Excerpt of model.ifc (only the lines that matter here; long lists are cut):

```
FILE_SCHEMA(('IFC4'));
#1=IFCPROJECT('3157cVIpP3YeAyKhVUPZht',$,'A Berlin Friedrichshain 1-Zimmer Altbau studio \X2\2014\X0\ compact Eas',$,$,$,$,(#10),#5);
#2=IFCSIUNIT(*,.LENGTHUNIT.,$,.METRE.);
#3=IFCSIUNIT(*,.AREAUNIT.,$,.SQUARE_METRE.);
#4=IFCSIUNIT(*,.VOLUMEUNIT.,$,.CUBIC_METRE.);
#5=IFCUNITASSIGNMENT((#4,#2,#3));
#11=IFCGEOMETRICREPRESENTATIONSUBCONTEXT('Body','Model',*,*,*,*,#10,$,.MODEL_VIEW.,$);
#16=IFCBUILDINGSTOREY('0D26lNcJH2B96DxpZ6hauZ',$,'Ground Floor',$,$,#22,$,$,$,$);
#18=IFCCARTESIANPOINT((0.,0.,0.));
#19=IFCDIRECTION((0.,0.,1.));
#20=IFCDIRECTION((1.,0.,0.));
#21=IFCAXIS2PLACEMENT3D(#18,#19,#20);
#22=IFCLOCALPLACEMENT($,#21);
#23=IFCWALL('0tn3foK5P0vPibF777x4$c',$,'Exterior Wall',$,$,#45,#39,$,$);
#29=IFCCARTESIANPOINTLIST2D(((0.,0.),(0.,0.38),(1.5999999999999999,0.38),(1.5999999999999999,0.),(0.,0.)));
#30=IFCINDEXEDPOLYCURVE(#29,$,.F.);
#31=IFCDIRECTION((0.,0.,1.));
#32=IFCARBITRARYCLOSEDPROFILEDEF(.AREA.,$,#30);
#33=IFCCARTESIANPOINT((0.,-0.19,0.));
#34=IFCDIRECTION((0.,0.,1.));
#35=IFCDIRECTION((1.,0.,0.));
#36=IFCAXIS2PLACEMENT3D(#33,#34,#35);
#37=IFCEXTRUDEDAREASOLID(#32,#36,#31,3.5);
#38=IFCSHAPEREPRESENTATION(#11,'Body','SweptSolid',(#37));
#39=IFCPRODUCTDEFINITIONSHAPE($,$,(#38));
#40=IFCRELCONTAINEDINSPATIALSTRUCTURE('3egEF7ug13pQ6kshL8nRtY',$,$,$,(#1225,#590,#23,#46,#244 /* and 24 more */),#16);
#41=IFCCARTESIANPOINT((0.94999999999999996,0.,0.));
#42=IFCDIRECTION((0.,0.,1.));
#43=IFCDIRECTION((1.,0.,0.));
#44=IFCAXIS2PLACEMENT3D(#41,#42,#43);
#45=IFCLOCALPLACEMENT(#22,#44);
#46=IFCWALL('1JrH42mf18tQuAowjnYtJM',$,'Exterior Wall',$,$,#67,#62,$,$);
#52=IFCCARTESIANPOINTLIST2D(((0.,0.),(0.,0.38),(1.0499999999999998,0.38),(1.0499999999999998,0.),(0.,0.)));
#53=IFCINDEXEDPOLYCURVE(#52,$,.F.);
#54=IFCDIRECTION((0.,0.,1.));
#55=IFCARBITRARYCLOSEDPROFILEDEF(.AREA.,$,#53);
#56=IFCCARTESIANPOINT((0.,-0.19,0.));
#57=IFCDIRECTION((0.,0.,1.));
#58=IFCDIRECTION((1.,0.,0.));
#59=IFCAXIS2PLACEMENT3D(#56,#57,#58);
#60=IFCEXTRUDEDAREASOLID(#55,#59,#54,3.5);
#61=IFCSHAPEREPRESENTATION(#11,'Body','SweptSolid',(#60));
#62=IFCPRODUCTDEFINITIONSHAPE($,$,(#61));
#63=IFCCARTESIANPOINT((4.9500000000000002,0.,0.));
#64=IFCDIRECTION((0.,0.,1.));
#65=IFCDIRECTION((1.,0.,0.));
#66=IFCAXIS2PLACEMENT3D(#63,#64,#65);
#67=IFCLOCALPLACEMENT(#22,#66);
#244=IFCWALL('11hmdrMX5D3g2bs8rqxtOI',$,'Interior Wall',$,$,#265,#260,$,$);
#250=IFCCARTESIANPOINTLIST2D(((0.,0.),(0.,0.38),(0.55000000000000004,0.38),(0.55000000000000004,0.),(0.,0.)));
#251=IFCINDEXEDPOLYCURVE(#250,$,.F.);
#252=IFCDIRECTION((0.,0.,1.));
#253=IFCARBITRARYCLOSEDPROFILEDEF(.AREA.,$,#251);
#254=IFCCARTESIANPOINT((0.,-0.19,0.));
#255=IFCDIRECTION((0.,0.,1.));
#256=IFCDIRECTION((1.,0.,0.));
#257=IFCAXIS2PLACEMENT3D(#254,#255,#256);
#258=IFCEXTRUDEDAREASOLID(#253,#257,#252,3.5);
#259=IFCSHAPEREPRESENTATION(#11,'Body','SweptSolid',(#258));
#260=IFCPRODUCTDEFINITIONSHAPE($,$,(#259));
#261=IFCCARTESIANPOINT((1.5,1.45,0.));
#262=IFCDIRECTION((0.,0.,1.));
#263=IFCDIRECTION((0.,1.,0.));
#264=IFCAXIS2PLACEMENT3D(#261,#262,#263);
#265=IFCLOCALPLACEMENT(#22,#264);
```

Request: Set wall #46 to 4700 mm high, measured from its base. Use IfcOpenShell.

```python
import ifcopenshell
import ifcopenshell.geom
import ifcopenshell.util.representation
import ifcopenshell.util.shape
import ifcopenshell.util.unit

model = ifcopenshell.open("model.ifc")
unit_scale = ifcopenshell.util.unit.calculate_unit_scale(model)
settings = ifcopenshell.geom.settings()


def volume(element):
    """Net volume in cubic metres, openings subtracted."""
    shape = ifcopenshell.geom.create_shape(settings, element)
    return ifcopenshell.util.shape.get_volume(shape.geometry)


wall = model.by_id(46)
before = volume(wall)

body = ifcopenshell.util.representation.get_representation(wall, "Model", "Body")
solid = body.Items[0]
old_height = solid.Depth
solid.Depth = 4.7 / unit_scale
after = volume(wall)

print(f"height {old_height:g} -> {solid.Depth:g}, volume {before:.3f} -> {after:.3f} m3")

model.write("model_updated.ifc")
```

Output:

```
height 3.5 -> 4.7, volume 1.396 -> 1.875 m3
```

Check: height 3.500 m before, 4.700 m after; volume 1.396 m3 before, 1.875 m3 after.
